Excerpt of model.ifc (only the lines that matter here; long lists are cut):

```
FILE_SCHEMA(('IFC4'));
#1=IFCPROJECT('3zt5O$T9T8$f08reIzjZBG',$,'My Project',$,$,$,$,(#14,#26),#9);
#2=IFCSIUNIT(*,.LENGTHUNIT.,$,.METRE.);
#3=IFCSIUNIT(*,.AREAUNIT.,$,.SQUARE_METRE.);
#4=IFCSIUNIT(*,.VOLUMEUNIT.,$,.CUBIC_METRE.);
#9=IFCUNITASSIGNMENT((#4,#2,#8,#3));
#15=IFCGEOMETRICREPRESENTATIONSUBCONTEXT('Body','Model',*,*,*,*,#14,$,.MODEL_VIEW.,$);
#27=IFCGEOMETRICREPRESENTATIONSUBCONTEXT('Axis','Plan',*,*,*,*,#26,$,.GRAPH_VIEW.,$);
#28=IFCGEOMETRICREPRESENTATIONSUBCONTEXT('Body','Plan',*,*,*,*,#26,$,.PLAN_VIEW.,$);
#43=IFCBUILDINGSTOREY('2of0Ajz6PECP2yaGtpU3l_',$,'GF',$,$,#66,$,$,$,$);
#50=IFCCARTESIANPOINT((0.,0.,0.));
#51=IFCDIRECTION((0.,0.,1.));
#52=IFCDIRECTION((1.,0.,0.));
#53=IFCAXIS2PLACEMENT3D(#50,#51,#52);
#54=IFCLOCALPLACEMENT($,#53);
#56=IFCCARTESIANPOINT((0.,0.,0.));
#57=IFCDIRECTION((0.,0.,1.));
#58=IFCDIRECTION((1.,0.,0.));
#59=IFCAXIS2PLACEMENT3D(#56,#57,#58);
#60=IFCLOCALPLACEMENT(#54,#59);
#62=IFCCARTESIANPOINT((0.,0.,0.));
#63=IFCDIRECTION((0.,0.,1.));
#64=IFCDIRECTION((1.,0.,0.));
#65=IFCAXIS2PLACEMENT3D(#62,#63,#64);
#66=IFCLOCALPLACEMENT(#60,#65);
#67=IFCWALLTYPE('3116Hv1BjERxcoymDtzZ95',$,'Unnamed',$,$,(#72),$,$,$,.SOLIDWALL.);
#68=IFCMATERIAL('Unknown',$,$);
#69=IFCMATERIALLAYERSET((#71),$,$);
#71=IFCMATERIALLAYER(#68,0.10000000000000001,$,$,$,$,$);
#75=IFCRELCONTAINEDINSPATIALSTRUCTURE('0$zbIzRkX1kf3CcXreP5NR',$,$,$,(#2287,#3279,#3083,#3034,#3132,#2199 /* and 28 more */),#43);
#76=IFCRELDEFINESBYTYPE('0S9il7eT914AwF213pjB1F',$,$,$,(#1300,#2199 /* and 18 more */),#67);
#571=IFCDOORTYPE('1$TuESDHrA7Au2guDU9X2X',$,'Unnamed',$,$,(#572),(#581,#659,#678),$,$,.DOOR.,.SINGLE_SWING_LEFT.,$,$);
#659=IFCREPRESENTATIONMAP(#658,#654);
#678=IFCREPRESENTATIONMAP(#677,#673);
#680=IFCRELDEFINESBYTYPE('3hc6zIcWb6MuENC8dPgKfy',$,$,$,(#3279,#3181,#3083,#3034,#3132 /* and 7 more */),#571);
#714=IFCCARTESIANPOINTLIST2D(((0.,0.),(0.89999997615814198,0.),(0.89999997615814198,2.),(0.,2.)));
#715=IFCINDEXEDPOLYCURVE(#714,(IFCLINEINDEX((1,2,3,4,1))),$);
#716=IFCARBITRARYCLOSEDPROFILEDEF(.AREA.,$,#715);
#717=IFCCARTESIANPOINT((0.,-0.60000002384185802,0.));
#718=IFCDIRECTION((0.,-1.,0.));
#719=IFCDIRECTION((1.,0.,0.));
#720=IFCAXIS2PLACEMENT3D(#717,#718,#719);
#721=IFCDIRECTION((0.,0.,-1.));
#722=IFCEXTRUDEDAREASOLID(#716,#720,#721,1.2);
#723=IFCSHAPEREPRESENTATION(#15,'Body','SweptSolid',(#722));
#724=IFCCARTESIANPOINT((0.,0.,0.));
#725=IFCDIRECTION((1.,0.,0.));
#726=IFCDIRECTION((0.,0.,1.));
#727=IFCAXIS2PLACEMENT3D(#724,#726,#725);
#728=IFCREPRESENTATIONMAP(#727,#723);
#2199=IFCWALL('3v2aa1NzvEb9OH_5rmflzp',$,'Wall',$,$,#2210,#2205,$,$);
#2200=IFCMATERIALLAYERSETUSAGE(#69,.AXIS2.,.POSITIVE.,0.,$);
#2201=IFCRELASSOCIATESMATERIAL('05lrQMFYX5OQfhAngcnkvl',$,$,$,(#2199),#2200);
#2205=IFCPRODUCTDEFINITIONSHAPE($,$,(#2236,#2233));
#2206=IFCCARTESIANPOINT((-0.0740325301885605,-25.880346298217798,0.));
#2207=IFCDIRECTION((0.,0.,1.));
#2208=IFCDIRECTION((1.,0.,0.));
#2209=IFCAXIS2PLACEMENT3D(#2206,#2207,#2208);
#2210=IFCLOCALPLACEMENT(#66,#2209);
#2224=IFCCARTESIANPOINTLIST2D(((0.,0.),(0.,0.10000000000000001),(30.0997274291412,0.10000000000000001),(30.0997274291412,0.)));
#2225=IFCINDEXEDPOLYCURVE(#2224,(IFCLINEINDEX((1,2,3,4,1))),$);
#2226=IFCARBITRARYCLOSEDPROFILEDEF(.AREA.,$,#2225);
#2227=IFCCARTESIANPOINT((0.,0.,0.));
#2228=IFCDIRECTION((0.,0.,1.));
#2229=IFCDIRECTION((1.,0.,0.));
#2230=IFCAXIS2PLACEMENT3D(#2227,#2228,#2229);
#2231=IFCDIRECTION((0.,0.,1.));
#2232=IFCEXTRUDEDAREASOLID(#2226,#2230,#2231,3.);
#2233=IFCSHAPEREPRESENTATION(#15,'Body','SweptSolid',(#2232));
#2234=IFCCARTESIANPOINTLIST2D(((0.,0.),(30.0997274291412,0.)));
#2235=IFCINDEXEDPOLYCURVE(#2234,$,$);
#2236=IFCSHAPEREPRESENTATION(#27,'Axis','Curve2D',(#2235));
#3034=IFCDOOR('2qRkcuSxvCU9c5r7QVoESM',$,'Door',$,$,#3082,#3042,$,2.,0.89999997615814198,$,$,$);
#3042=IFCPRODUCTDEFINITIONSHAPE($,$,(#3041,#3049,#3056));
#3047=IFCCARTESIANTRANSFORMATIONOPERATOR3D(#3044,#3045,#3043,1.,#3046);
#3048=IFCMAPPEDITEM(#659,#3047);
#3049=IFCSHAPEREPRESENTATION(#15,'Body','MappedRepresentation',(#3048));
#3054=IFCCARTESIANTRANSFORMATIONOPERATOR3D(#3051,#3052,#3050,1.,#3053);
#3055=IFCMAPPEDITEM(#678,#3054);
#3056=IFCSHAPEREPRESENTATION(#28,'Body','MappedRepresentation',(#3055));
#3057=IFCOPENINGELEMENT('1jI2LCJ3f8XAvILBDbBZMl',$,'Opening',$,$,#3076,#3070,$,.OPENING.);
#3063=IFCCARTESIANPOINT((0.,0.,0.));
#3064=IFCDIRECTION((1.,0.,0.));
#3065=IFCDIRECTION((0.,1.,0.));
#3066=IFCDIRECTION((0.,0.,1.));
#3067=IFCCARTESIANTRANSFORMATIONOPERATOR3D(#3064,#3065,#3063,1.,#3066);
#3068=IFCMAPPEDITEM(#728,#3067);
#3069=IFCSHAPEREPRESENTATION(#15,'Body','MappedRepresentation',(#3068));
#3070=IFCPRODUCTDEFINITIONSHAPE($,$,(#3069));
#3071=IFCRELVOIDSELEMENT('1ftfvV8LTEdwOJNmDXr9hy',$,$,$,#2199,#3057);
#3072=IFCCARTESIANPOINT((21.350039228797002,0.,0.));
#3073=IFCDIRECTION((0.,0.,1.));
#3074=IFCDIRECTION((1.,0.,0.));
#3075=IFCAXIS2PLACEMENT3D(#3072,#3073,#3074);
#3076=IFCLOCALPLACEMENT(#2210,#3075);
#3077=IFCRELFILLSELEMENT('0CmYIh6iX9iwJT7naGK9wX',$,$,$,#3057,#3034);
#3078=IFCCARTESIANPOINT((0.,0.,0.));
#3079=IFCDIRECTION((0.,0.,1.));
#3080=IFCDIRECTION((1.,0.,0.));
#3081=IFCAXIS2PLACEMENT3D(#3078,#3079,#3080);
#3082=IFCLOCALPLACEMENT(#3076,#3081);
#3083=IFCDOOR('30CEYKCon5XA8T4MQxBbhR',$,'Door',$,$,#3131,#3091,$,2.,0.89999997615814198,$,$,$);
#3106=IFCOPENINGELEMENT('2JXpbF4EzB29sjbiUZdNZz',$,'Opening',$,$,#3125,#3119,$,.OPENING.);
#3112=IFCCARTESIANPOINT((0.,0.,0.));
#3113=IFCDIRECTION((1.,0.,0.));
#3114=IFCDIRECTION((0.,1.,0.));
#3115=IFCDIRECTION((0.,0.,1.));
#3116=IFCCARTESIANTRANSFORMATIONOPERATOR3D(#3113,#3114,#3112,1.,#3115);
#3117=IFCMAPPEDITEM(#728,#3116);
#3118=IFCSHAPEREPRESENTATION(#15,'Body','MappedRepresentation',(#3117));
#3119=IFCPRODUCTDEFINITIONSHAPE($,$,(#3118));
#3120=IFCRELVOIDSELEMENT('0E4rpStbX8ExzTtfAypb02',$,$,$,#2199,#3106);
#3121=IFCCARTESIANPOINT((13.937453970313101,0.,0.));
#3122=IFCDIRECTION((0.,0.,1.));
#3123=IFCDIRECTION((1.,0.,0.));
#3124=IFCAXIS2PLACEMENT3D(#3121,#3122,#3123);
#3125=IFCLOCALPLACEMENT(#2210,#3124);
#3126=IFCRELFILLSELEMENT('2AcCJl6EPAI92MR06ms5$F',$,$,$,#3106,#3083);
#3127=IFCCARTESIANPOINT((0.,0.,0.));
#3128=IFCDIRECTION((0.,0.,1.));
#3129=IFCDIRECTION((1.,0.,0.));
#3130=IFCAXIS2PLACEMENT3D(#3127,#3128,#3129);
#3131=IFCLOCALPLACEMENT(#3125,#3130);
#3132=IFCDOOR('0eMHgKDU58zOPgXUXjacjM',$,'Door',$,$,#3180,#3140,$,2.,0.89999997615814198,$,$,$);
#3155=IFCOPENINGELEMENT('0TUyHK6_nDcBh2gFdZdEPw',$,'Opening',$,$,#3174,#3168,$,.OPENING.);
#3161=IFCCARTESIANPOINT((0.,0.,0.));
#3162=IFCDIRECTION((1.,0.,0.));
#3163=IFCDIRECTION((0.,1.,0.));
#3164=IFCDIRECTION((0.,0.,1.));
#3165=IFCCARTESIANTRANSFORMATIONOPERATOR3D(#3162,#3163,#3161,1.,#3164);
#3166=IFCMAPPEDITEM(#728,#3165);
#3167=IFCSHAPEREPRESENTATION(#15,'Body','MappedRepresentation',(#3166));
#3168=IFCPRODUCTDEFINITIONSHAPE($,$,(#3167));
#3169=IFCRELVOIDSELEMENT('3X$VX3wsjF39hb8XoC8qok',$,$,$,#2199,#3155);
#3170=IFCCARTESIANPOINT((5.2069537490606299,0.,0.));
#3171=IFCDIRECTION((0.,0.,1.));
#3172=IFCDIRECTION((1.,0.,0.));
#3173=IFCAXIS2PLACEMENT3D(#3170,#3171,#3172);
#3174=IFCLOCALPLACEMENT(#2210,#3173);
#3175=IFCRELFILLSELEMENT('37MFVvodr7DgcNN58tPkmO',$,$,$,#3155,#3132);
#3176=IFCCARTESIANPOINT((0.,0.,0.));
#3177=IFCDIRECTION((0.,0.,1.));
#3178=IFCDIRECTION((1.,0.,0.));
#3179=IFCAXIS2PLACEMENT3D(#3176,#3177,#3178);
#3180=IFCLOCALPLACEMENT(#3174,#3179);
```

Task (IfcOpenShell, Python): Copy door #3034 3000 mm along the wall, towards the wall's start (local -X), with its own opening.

```python
import ifcopenshell
import ifcopenshell.api.feature
import ifcopenshell.api.geometry
import ifcopenshell.api.root
import ifcopenshell.geom
import ifcopenshell.util.element
import ifcopenshell.util.placement
import ifcopenshell.util.shape
import ifcopenshell.util.unit

model = ifcopenshell.open("model.ifc")
unit_scale = ifcopenshell.util.unit.calculate_unit_scale(model)
settings = ifcopenshell.geom.settings()


def volume(element):
    """Net volume in cubic metres, openings subtracted."""
    shape = ifcopenshell.geom.create_shape(settings, element)
    return ifcopenshell.util.shape.get_volume(shape.geometry)


door = model.by_guid("2qRkcuSxvCU9c5r7QVoESM")
opening = door.FillsVoids[0].RelatingOpeningElement
wall = opening.VoidsElements[0].RelatingBuildingElement
before = volume(wall)
shift = ifcopenshell.util.placement.get_local_placement(wall.ObjectPlacement)[:3, 0] * -3 / unit_scale

# copy_class copies the void relationship, type, container and properties, but no geometry.
new_opening = ifcopenshell.api.root.copy_class(model, product=opening)
new_opening.Representation = ifcopenshell.util.element.copy_deep(
    model, opening.Representation, exclude=["IfcGeometricRepresentationContext", "IfcRepresentationMap"]
)
new_door = ifcopenshell.api.root.copy_class(model, product=door)
new_door.Representation = ifcopenshell.util.element.copy_deep(
    model, door.Representation, exclude=["IfcGeometricRepresentationContext", "IfcRepresentationMap"]
)
ifcopenshell.api.feature.add_filling(model, opening=new_opening, element=new_door)

for old, new in ((opening, new_opening), (door, new_door)):
    matrix = ifcopenshell.util.placement.get_local_placement(old.ObjectPlacement)
    matrix[:3, 3] += shift
    ifcopenshell.api.geometry.edit_object_placement(model, product=new, matrix=matrix, is_si=False)

after = volume(wall)

print(f"wall volume {before:.3f} -> {after:.3f} m3")

model.write("model-out.ifc")
```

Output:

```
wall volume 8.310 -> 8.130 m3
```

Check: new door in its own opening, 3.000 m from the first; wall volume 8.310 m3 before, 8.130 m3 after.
